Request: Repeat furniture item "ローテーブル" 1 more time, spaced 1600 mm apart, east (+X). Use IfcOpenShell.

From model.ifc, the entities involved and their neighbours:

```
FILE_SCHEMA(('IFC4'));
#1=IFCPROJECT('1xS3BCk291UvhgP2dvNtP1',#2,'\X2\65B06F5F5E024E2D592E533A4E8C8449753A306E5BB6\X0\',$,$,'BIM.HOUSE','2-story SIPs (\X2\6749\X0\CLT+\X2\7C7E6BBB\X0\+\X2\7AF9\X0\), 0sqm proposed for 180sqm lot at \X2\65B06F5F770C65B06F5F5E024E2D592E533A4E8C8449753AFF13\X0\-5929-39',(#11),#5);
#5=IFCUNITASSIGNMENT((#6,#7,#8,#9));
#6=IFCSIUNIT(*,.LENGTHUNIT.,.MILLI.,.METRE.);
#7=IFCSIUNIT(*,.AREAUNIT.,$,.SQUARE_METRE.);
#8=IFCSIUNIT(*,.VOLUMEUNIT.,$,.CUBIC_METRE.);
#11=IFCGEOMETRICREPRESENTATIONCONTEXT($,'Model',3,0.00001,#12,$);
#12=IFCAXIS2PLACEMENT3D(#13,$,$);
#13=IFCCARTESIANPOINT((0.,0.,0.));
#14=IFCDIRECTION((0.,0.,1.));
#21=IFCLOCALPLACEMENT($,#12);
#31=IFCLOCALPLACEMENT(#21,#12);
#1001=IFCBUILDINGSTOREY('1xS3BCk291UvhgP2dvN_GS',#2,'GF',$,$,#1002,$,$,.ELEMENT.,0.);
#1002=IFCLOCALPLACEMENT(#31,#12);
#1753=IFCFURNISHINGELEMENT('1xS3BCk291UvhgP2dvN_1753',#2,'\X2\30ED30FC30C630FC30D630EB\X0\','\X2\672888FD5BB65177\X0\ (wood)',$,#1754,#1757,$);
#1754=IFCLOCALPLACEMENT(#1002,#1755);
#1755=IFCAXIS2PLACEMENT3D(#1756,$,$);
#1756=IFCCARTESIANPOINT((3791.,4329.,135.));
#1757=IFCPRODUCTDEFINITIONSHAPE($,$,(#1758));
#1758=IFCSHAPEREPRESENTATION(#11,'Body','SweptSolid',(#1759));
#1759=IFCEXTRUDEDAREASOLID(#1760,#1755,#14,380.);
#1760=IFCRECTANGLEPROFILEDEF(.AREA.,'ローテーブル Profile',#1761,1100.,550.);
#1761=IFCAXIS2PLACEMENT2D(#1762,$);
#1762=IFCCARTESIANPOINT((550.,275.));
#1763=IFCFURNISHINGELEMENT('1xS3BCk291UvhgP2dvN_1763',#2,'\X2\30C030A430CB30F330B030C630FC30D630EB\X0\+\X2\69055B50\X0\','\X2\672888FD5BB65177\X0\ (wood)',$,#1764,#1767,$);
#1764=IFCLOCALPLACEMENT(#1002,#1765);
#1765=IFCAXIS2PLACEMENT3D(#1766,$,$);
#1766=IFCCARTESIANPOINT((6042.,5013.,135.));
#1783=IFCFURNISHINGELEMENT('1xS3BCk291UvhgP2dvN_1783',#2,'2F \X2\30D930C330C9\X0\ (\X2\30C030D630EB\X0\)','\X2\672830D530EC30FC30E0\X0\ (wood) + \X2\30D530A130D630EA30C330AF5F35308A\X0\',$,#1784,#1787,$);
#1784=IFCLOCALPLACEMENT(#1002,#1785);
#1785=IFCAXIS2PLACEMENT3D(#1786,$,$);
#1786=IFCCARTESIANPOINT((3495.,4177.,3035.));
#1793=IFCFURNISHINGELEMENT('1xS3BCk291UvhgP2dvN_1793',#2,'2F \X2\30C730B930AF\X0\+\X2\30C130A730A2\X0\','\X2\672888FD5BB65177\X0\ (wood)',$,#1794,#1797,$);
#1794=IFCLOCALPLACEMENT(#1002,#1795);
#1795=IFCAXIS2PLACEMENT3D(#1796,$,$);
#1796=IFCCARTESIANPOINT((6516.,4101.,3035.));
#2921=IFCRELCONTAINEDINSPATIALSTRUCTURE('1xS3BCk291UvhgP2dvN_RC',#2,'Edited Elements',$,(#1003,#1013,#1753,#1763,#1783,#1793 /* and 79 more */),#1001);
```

```python
import numpy as np
import ifcopenshell
import ifcopenshell.api.geometry
import ifcopenshell.api.root
import ifcopenshell.util.element
import ifcopenshell.util.placement

model = ifcopenshell.open("model.ifc")


def reuse_history(source, copy):
    """copy_class also copies each property set's owner history, people and application; keep the originals."""
    for rel in copy.IsDefinedBy:
        if rel.is_a("IfcRelDefinesByProperties") and (history := rel.RelatingPropertyDefinition.OwnerHistory):
            rel.RelatingPropertyDefinition.OwnerHistory = source.OwnerHistory
            ifcopenshell.util.element.remove_deep2(model, history)


source = model.by_id(1753)
base = ifcopenshell.util.placement.get_local_placement(source.ObjectPlacement)
step = np.array([1.0, 0.0, 0.0]) * 1600.0

for i in range(1, 2):
    copy = ifcopenshell.api.root.copy_class(model, product=source)
    copy.Representation = ifcopenshell.util.element.copy_deep(
        model, source.Representation, exclude=["IfcGeometricRepresentationContext", "IfcRepresentationMap"]
    )
    reuse_history(source, copy)
    matrix = base.copy()
    matrix[:3, 3] += i * step
    print("added at", matrix[:3, 3].round(3) + 0.0)
    ifcopenshell.api.geometry.edit_object_placement(model, product=copy, matrix=matrix, is_si=False)

model.write("model_edited.ifc")
```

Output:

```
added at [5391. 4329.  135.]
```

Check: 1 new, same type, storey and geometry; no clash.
